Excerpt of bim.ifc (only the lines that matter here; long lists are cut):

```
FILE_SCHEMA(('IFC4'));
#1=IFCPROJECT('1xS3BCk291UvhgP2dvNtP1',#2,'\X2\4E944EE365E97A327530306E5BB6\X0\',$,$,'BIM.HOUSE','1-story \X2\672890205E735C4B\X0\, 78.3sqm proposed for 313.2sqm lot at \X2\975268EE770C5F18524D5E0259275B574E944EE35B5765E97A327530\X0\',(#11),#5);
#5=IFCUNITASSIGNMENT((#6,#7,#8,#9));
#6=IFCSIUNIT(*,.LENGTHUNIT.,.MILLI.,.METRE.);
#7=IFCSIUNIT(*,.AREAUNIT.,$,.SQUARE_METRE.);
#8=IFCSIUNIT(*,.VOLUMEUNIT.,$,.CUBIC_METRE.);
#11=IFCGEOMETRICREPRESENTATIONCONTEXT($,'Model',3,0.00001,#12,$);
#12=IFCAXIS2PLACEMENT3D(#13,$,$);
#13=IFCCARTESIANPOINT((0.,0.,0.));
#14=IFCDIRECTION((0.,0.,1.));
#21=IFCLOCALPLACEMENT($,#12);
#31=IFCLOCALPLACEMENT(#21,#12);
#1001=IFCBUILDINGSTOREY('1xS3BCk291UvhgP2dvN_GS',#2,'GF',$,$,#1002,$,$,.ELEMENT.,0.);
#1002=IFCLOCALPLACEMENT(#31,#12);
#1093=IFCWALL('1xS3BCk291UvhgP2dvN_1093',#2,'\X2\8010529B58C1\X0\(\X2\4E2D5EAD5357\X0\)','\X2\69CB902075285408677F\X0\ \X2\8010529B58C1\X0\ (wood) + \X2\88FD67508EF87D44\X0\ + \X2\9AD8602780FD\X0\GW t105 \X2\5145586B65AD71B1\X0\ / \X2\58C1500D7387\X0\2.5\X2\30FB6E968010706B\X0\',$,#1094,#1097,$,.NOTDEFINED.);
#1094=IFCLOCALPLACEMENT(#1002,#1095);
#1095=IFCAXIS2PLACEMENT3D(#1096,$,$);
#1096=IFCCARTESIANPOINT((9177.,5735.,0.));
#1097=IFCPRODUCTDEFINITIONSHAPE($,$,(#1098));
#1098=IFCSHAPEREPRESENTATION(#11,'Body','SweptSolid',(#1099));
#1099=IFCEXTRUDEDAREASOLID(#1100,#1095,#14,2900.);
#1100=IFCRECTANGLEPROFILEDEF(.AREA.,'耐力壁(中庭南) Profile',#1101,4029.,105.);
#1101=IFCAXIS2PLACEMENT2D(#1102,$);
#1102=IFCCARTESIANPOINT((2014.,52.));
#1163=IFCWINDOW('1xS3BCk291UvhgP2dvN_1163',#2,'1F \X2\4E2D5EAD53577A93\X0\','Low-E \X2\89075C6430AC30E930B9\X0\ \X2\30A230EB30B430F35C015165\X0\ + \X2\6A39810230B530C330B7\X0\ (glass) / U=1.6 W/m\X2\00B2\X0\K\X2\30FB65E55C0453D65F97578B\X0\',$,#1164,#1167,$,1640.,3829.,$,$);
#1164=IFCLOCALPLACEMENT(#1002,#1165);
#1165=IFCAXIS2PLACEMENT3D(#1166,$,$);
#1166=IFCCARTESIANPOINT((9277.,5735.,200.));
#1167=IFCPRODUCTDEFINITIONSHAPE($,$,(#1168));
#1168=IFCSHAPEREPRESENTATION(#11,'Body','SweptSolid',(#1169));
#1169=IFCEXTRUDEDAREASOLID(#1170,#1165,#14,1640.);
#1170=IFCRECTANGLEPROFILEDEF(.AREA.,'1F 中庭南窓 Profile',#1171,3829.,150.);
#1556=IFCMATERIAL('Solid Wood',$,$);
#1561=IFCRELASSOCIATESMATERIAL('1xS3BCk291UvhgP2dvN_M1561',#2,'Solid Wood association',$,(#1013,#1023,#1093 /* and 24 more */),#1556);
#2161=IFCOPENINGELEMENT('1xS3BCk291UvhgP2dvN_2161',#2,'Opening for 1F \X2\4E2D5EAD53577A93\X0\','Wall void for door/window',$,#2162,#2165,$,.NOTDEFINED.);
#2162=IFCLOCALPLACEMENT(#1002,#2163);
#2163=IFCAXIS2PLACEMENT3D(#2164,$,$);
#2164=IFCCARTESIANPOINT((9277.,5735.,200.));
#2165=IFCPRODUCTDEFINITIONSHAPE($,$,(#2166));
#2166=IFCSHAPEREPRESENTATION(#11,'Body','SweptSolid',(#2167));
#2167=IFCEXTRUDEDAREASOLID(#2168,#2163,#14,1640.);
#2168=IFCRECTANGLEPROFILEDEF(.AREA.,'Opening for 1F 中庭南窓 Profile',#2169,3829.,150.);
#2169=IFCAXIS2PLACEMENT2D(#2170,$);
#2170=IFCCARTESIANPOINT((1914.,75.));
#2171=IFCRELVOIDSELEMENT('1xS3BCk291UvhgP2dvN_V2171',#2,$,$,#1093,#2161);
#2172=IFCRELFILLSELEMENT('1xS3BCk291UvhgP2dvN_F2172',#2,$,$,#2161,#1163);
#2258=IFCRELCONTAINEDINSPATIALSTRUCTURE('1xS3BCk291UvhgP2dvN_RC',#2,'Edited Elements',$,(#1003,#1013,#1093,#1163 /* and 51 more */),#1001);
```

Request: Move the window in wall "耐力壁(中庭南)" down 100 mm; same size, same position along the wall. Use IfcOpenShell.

```python
import numpy as np
import ifcopenshell
import ifcopenshell.api.geometry
import ifcopenshell.util.placement
import ifcopenshell.util.unit

model = ifcopenshell.open("bim.ifc")
unit_scale = ifcopenshell.util.unit.calculate_unit_scale(model)

window = model.by_id(1163)
opening = window.FillsVoids[0].RelatingOpeningElement
dz = -0.1 / unit_scale

shift = np.array([0.0, 0.0, dz])
# The window is not placed relative to its opening, so move both.
for product in (opening, window):
    matrix = ifcopenshell.util.placement.get_local_placement(product.ObjectPlacement)
    matrix[:3, 3] += shift
    ifcopenshell.api.geometry.edit_object_placement(model, product=product, matrix=matrix, is_si=False)

print(f"moved by {dz * unit_scale:+.3f} m")

model.write("bim-out.ifc")
```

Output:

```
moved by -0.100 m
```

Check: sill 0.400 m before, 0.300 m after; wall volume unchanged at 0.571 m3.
